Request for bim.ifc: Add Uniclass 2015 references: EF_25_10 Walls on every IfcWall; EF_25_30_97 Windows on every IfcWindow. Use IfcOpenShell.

First a look at what the model holds.

```python
import ifcopenshell

model = ifcopenshell.open("bim.ifc")
print(model.schema)
print("classifications:", [c.Name for c in model.by_type("IfcClassification")])
for ifc_class in ("IfcDoor", "IfcRoof", "IfcStair", "IfcWall", "IfcWindow"):
    print(ifc_class, len(model.by_type(ifc_class)))
```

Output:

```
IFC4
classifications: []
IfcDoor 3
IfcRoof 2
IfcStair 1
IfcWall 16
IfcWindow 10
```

```python
import ifcopenshell
import ifcopenshell.api.classification

model = ifcopenshell.open("bim.ifc")

system = ifcopenshell.api.classification.add_classification(model, classification="Uniclass 2015")

codes = {
    "IfcWall": ("EF_25_10", "Walls"),
    "IfcWindow": ("EF_25_30_97", "Windows"),
}
for ifc_class, (code, name) in codes.items():
    products = model.by_type(ifc_class)
    ifcopenshell.api.classification.add_reference(
        model, products=products, classification=system, identification=code, name=name
    )
    print(code, len(products))

model.write("bim-out.ifc")
```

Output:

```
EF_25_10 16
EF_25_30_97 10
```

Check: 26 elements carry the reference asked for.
